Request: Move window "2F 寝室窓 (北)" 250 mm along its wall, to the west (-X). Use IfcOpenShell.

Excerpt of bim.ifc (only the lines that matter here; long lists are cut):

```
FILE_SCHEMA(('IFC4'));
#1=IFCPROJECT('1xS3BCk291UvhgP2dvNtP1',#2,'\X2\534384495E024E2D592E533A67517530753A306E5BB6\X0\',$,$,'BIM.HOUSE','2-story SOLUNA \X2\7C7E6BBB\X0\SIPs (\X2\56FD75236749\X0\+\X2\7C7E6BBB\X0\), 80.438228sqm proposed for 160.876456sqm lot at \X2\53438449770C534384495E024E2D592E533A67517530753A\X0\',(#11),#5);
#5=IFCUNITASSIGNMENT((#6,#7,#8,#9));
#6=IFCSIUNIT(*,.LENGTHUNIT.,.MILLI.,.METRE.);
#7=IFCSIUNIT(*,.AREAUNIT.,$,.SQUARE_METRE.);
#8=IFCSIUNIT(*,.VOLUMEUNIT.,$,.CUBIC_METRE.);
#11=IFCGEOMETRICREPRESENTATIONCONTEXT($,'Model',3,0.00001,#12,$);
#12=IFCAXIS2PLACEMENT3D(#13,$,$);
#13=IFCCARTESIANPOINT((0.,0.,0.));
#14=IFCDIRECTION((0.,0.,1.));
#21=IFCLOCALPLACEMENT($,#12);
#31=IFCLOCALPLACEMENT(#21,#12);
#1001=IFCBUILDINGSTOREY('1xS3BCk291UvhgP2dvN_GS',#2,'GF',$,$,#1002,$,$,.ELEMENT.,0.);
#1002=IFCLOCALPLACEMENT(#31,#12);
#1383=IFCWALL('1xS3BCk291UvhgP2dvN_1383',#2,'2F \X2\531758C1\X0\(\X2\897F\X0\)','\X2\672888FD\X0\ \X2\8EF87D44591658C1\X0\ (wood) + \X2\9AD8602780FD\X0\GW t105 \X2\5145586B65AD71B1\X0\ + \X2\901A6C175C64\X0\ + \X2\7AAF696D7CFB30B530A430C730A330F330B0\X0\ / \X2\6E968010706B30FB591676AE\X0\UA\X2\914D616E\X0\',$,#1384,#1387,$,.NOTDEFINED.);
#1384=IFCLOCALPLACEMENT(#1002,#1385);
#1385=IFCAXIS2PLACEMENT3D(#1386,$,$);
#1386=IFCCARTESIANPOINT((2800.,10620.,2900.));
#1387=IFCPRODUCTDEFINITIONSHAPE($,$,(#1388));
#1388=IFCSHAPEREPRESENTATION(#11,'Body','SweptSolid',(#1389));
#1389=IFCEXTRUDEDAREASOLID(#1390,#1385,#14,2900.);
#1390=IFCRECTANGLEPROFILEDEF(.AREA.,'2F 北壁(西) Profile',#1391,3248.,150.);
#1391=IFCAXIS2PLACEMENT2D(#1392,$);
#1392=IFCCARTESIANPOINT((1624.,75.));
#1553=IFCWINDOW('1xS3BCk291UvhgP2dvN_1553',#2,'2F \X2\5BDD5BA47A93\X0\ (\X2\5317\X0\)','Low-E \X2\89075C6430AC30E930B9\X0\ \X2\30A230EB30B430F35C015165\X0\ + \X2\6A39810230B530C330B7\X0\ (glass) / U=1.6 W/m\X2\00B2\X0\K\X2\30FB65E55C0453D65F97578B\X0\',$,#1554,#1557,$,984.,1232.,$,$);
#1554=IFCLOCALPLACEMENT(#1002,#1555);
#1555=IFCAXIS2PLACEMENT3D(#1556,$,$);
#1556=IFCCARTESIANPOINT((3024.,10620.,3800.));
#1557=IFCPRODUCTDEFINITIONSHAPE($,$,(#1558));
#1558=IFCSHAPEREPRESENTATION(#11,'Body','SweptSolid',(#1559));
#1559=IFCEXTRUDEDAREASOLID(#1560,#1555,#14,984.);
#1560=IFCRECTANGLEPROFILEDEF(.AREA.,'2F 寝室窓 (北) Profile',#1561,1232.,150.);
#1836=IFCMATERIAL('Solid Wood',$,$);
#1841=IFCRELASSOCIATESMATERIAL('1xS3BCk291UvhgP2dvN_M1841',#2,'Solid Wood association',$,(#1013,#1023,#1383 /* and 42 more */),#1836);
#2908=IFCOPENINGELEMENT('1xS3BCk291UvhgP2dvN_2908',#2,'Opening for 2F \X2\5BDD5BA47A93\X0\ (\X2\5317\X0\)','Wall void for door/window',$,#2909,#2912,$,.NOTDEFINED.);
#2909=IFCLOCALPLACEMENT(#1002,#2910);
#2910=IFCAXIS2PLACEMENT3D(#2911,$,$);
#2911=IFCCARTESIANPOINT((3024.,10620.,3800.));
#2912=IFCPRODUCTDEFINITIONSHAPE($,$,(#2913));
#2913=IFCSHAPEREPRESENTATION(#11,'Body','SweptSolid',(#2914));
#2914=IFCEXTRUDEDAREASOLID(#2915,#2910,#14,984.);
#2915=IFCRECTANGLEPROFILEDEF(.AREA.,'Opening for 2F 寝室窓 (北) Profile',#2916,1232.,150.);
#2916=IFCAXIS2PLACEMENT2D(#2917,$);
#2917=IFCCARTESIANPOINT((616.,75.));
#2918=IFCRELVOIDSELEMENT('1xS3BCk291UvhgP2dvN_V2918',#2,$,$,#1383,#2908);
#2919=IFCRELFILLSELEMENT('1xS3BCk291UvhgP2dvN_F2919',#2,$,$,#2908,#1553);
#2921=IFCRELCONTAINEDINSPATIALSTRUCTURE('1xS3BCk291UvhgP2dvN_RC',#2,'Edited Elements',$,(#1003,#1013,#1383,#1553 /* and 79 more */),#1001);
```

```python
import ifcopenshell
import ifcopenshell.api.geometry
import ifcopenshell.util.placement
import ifcopenshell.util.unit

model = ifcopenshell.open("bim.ifc")
unit_scale = ifcopenshell.util.unit.calculate_unit_scale(model)

window = model.by_guid("1xS3BCk291UvhgP2dvN_1553")
opening = window.FillsVoids[0].RelatingOpeningElement
wall = opening.VoidsElements[0].RelatingBuildingElement

wall_matrix = ifcopenshell.util.placement.get_local_placement(wall.ObjectPlacement)
shift = wall_matrix[:3, 0] * -0.25 / unit_scale
before = ifcopenshell.util.placement.get_local_placement(window.ObjectPlacement)[:3, 3].copy()

# The window is not placed relative to its opening, so move both.
for product in (opening, window):
    matrix = ifcopenshell.util.placement.get_local_placement(product.ObjectPlacement)
    matrix[:3, 3] += shift
    ifcopenshell.api.geometry.edit_object_placement(model, product=product, matrix=matrix, is_si=False)

after = ifcopenshell.util.placement.get_local_placement(window.ObjectPlacement)[:3, 3]
print("window moved by", (after - before).round(3) + 0.0)

model.write("bim_v2.ifc")
```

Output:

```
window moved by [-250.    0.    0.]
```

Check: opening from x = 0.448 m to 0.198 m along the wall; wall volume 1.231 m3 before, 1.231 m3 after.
